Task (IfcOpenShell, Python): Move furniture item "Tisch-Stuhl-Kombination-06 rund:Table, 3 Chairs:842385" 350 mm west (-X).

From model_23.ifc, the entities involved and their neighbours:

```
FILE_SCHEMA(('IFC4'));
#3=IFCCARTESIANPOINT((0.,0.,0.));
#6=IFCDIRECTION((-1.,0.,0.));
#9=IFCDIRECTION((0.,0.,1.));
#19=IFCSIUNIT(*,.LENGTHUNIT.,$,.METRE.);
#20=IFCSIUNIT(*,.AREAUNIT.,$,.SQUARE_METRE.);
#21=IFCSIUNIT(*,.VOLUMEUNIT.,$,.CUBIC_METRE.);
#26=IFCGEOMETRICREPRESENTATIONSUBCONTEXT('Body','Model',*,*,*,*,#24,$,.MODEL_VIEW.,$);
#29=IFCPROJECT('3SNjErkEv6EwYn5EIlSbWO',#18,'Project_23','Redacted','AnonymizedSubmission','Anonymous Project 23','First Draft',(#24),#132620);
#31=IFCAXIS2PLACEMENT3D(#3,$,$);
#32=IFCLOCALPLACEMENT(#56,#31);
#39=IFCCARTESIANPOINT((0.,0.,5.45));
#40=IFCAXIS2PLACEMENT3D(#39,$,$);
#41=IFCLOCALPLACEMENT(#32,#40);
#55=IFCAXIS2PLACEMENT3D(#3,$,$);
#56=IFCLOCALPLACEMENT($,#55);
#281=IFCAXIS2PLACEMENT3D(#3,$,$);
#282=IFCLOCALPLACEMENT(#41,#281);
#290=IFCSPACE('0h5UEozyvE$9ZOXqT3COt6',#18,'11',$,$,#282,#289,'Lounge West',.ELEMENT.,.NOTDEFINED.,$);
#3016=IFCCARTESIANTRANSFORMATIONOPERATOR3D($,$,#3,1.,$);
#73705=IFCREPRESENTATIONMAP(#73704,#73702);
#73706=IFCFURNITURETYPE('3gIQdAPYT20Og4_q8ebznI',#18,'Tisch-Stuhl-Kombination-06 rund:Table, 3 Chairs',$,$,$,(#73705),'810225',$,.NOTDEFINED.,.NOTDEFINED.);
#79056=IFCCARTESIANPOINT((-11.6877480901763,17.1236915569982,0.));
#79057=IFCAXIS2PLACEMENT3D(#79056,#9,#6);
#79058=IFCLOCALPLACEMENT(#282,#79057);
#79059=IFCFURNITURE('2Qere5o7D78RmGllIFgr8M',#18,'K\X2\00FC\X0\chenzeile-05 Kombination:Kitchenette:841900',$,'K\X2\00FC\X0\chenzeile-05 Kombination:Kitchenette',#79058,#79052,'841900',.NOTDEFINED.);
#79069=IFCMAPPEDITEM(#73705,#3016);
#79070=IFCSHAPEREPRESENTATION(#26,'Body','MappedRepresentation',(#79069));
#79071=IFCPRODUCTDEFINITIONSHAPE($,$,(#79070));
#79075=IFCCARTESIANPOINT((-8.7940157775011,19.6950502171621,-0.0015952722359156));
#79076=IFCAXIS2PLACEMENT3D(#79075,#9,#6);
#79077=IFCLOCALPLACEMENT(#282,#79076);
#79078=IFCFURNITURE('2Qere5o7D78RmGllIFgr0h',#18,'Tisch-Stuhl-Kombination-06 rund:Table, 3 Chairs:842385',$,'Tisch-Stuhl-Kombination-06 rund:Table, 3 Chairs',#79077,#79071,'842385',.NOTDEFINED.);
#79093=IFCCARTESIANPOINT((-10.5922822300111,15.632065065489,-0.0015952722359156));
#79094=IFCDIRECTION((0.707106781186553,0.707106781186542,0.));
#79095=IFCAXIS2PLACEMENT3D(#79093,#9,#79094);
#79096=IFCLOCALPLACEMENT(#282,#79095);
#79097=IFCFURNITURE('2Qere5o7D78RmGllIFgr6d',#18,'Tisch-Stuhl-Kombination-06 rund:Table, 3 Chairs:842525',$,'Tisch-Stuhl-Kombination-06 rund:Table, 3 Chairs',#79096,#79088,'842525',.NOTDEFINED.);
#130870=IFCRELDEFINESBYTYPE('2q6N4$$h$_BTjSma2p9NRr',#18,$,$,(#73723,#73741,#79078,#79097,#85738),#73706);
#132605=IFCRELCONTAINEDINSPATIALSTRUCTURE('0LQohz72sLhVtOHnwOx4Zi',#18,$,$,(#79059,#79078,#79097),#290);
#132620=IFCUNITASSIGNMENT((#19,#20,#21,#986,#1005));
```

```python
import ifcopenshell
import ifcopenshell.api.geometry
import ifcopenshell.util.placement

model = ifcopenshell.open("model_23.ifc")

item = model.by_guid("2Qere5o7D78RmGllIFgr0h")
matrix = ifcopenshell.util.placement.get_local_placement(item.ObjectPlacement)
matrix[0, 3] -= 0.35
ifcopenshell.api.geometry.edit_object_placement(model, product=item, matrix=matrix, is_si=False)

print(ifcopenshell.util.placement.get_local_placement(item.ObjectPlacement).round(3) + 0.0)

model.write("model_23_updated.ifc")
```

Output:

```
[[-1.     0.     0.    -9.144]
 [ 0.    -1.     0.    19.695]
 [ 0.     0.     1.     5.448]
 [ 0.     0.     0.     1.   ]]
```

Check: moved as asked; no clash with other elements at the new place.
